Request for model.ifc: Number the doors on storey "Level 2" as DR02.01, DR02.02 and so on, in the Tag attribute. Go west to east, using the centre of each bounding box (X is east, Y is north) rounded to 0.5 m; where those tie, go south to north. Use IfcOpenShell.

First a look at what the model holds.

```python
import ifcopenshell
import ifcopenshell.util.element
import ifcopenshell.util.placement

model = ifcopenshell.open("model.ifc")
print(model.schema)
storey = next(s for s in model.by_type("IfcBuildingStorey") if s.Name == "Level 2")
doors = [e for e in ifcopenshell.util.element.get_decomposition(storey) if e.is_a("IfcDoor")]
for e in sorted(doors, key=lambda e: e.id()):
    origin = ifcopenshell.util.placement.get_local_placement(e.ObjectPlacement)[:3, 3]
    print(e.id(), e.Tag, e.Name, origin.round(2) + 0.0, sep=" | ")
```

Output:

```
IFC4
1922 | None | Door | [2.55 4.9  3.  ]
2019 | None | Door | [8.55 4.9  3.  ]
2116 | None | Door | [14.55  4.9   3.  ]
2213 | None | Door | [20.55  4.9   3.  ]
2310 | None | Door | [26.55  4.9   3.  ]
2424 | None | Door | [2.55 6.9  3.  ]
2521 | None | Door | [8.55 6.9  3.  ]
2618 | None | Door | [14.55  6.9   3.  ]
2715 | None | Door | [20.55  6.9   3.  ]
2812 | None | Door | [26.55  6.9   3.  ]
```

```python
import ifcopenshell
import ifcopenshell.geom
import ifcopenshell.util.element
import ifcopenshell.util.shape

model = ifcopenshell.open("model.ifc")
settings = ifcopenshell.geom.settings()
settings.set("use-world-coords", True)


def centre(element):
    shape = ifcopenshell.geom.create_shape(settings, element)
    return ifcopenshell.util.shape.get_bbox_centroid(shape.geometry)


storey = next(s for s in model.by_type("IfcBuildingStorey") if s.Name == "Level 2")
doors = [e for e in ifcopenshell.util.element.get_decomposition(storey) if e.is_a("IfcDoor")]

# Insertion points can sit at a corner or the storey origin, so sort by the geometry (in metres).
centres = {e: centre(e) for e in doors}
doors.sort(key=lambda e: (round(centres[e][0] / 0.5), centres[e][1]))

for i, e in enumerate(doors, start=1):
    number = f"DR02.{i:02d}"
    e.Tag = number
    print(e.id(), number)

model.write("model-out.ifc")
```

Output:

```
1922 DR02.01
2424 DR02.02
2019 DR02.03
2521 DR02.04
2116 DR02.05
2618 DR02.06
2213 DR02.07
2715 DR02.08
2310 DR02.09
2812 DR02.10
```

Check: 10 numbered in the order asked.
